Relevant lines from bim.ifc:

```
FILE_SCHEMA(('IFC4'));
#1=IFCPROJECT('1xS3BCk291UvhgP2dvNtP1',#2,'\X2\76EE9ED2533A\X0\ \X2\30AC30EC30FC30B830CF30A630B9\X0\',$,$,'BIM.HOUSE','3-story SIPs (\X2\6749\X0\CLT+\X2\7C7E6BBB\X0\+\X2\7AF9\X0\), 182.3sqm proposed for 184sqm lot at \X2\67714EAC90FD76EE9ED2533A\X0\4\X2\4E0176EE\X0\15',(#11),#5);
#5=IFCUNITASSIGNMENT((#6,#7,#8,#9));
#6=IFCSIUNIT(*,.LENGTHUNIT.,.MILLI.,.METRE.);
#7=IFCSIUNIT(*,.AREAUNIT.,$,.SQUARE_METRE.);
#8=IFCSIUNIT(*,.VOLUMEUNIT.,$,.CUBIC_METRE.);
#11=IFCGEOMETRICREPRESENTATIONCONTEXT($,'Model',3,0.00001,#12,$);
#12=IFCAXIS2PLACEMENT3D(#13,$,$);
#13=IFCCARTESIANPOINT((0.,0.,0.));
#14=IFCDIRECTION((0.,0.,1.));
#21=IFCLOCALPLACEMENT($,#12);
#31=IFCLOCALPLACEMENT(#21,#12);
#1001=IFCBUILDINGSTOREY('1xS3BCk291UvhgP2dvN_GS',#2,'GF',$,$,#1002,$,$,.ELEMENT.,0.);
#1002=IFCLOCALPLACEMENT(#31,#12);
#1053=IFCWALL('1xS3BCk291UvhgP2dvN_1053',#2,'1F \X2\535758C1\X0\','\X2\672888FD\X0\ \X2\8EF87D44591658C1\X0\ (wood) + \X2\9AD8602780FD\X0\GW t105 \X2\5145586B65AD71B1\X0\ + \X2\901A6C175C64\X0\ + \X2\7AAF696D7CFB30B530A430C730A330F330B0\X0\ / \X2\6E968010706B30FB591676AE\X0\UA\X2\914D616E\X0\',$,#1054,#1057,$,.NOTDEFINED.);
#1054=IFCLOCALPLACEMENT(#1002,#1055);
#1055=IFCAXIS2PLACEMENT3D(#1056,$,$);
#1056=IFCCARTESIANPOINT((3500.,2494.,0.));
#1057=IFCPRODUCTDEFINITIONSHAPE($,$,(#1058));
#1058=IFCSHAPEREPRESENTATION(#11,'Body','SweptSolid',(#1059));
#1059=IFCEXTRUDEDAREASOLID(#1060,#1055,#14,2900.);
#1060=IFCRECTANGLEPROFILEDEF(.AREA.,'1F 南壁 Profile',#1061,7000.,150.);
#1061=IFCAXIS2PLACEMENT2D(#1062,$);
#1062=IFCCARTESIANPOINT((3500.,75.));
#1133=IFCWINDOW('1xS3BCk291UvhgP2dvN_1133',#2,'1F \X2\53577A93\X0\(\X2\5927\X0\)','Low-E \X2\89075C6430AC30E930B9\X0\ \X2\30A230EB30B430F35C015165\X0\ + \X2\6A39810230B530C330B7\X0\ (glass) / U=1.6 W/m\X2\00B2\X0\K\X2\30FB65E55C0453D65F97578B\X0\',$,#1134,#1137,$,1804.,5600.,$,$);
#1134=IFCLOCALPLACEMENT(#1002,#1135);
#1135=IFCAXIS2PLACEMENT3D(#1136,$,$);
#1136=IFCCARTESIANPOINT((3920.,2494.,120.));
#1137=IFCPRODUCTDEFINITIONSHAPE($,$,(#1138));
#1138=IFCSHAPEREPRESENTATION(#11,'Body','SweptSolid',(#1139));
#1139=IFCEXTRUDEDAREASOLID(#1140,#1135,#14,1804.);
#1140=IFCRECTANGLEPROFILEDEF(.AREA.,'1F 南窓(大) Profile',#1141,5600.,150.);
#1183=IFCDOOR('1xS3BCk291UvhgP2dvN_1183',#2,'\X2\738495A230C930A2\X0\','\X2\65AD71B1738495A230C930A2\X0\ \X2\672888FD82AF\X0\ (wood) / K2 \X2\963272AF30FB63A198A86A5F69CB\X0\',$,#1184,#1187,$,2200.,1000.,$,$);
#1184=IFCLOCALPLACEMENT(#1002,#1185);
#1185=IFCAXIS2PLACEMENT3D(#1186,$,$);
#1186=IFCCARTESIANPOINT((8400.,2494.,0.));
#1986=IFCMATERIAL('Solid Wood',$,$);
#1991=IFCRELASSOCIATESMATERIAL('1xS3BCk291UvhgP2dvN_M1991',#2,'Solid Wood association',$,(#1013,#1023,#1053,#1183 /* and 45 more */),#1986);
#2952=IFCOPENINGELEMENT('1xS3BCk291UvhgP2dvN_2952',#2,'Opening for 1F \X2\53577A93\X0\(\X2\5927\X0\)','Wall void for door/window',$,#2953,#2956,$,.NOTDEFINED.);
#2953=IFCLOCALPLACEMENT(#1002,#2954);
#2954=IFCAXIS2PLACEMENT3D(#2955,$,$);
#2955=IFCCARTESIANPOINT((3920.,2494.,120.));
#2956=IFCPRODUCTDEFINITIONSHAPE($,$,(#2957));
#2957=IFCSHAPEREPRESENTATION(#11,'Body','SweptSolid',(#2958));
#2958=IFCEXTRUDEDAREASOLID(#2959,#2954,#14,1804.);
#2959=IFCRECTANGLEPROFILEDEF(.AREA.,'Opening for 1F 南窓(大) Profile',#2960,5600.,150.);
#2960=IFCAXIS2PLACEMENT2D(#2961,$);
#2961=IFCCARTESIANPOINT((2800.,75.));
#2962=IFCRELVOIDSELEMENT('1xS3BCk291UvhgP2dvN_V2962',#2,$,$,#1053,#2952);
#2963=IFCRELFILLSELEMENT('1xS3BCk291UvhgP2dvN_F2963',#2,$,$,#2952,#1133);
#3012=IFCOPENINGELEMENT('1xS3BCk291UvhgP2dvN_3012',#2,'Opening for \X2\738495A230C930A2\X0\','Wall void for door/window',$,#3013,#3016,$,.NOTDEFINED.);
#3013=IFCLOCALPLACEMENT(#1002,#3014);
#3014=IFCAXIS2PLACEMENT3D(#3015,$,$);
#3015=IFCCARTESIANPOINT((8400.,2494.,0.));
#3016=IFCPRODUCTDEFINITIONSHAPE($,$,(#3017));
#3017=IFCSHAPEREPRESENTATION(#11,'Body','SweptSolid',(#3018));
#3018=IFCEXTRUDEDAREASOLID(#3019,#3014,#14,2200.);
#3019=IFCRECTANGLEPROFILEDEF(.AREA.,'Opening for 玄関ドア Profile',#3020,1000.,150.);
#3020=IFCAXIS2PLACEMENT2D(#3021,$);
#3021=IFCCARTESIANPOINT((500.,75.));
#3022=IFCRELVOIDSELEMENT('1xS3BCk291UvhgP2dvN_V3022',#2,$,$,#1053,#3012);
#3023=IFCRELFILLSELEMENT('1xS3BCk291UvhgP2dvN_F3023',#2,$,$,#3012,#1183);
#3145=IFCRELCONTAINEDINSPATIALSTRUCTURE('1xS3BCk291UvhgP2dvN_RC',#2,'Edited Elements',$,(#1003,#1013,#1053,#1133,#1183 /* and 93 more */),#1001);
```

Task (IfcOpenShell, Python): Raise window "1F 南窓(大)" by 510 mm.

```python
import numpy as np
import ifcopenshell
import ifcopenshell.api.geometry
import ifcopenshell.util.placement
import ifcopenshell.util.unit

model = ifcopenshell.open("bim.ifc")
unit_scale = ifcopenshell.util.unit.calculate_unit_scale(model)

window = model.by_guid("1xS3BCk291UvhgP2dvN_1133")
opening = window.FillsVoids[0].RelatingOpeningElement
dz = 0.51 / unit_scale

shift = np.array([0.0, 0.0, dz])
# The window is not placed relative to its opening, so move both.
for product in (opening, window):
    matrix = ifcopenshell.util.placement.get_local_placement(product.ObjectPlacement)
    matrix[:3, 3] += shift
    ifcopenshell.api.geometry.edit_object_placement(model, product=product, matrix=matrix, is_si=False)

print(f"moved by {dz * unit_scale:+.3f} m")

model.write("bim_v2.ifc")
```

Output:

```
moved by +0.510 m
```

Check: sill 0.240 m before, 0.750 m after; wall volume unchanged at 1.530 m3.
